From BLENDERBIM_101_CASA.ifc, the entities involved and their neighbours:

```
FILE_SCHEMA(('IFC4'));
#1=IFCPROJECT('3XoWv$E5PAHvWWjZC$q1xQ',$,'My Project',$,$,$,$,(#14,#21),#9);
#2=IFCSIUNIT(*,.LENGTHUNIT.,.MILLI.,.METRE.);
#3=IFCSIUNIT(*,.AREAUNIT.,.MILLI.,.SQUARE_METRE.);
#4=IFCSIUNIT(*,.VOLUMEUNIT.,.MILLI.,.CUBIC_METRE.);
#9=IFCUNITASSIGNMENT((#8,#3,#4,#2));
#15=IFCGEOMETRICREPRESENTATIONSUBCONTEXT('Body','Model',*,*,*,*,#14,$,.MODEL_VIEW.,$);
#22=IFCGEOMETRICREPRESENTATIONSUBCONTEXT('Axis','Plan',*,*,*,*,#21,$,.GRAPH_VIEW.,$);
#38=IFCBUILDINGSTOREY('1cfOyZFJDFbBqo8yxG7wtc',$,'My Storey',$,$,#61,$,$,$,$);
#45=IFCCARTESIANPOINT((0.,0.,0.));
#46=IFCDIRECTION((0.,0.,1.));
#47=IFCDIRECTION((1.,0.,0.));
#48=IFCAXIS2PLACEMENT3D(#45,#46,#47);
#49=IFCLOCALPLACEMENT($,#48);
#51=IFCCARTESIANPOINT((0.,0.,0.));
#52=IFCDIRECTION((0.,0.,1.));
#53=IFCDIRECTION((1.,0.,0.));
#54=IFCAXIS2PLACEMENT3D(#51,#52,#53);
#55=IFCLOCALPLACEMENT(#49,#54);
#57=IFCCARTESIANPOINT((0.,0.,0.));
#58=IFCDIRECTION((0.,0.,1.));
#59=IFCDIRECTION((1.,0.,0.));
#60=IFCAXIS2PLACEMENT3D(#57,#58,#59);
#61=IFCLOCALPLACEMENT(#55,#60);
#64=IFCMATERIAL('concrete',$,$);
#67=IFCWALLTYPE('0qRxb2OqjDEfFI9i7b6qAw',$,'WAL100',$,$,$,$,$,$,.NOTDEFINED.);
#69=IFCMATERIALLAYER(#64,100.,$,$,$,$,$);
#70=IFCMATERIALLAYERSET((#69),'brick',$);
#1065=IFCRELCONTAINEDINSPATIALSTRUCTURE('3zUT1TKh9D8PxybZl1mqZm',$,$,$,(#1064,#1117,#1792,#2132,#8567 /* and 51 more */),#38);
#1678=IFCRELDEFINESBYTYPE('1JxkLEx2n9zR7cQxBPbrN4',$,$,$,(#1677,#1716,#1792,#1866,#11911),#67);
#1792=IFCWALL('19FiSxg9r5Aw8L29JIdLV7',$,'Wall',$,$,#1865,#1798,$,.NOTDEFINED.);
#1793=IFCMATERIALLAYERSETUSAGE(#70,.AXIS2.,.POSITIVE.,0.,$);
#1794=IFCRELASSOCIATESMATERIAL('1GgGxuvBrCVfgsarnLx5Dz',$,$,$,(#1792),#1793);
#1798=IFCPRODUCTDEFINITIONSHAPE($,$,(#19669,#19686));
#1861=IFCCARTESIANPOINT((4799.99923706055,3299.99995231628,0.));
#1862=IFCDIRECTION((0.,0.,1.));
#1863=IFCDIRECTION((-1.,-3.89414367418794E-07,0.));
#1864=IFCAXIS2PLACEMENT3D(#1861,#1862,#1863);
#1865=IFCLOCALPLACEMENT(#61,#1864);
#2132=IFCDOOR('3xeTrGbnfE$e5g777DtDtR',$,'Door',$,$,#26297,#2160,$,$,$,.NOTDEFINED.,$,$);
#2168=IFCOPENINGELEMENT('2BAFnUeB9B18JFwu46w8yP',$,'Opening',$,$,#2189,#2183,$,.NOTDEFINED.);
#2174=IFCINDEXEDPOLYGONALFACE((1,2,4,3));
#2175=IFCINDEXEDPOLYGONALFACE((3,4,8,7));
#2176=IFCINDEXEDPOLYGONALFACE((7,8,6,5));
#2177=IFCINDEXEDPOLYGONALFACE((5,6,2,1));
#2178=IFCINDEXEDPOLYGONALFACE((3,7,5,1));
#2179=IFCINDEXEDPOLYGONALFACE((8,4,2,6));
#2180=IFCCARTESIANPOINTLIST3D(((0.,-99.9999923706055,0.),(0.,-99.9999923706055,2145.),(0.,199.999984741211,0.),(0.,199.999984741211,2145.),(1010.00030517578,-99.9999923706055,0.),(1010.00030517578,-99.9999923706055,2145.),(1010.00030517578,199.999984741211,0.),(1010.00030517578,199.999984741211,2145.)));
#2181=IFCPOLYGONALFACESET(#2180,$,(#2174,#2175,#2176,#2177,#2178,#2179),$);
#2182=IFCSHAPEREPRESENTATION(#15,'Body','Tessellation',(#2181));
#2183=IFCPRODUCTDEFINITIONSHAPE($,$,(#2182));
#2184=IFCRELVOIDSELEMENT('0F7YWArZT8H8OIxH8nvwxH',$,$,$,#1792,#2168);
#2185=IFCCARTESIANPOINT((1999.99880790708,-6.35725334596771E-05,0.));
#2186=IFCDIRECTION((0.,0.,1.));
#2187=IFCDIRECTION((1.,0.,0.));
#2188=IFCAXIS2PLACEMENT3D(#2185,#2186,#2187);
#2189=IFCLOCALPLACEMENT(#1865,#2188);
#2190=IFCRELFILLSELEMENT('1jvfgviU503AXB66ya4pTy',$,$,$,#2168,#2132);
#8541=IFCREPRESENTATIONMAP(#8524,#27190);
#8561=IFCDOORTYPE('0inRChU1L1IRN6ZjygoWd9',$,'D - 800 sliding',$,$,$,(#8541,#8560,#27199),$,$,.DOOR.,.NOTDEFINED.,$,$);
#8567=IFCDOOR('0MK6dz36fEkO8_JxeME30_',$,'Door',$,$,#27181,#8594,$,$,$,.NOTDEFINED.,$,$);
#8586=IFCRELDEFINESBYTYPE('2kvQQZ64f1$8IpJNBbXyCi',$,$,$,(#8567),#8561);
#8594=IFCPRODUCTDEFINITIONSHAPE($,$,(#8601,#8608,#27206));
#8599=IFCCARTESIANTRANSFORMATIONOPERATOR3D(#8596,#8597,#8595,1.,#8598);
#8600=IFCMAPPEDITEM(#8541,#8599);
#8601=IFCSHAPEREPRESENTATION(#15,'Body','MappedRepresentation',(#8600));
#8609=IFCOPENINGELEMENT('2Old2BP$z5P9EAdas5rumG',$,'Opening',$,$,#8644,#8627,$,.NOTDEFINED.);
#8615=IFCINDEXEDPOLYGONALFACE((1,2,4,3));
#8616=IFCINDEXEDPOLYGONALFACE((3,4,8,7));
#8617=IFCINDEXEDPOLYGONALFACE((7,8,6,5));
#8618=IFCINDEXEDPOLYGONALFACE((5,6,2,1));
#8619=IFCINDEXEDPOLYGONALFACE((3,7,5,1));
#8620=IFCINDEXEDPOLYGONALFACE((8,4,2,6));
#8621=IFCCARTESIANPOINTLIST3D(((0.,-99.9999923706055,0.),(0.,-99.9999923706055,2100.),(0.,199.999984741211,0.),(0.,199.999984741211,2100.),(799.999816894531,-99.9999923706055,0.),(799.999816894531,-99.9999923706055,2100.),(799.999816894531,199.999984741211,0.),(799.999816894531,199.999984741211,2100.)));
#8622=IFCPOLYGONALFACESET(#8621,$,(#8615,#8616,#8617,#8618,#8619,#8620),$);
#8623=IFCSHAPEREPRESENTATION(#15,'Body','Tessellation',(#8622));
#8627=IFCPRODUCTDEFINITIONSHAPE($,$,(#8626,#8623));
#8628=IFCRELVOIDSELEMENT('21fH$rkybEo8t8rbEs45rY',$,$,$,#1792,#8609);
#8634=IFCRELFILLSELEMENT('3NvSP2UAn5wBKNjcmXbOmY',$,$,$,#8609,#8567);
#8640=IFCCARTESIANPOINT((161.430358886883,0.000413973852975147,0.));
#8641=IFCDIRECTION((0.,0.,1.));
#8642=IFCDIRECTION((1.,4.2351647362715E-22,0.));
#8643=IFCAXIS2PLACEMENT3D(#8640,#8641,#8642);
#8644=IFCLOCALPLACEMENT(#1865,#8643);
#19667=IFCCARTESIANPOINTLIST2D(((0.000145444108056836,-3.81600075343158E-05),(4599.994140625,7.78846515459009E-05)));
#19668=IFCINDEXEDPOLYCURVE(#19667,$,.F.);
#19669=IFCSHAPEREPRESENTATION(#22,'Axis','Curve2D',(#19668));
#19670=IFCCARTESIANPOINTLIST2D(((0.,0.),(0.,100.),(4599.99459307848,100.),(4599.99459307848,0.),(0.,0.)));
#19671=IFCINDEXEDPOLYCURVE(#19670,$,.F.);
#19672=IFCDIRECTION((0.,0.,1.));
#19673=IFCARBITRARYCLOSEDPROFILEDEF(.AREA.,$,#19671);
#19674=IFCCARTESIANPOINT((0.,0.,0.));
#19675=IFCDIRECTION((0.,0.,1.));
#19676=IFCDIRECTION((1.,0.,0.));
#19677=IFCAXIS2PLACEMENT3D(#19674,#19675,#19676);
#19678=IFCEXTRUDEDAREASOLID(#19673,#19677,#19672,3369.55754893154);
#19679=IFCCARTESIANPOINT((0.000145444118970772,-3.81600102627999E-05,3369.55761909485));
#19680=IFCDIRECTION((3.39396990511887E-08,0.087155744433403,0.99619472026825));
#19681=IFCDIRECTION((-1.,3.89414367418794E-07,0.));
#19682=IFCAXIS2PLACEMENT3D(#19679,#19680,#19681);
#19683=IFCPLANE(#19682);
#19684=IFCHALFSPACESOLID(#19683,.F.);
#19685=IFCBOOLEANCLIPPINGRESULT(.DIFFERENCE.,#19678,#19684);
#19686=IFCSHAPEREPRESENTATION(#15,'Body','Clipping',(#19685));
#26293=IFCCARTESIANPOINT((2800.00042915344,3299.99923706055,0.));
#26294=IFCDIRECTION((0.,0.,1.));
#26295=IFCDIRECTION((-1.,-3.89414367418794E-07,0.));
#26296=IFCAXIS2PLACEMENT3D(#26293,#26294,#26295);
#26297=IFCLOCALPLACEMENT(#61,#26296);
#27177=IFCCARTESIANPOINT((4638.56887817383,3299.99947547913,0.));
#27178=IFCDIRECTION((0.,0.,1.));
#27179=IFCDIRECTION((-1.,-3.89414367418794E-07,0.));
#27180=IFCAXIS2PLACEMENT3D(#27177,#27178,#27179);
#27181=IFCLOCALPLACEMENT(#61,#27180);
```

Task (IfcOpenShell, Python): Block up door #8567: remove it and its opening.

```python
import ifcopenshell
import ifcopenshell.api.feature
import ifcopenshell.api.root
import ifcopenshell.geom
import ifcopenshell.util.shape

model = ifcopenshell.open("BLENDERBIM_101_CASA.ifc")
settings = ifcopenshell.geom.settings()


def volume(element):
    """Net volume in cubic metres, openings subtracted."""
    shape = ifcopenshell.geom.create_shape(settings, element)
    return ifcopenshell.util.shape.get_volume(shape.geometry)


door = model.by_guid("0MK6dz36fEkO8_JxeME30_")
opening = door.FillsVoids[0].RelatingOpeningElement
wall = opening.VoidsElements[0].RelatingBuildingElement
before = volume(wall)

ifcopenshell.api.root.remove_product(model, product=door)
ifcopenshell.api.feature.remove_feature(model, feature=opening)

after = volume(wall)

print(f"wall volume {before:.3f} -> {after:.3f} m3")

model.write("BLENDERBIM_101_CASA_edited.ifc")
```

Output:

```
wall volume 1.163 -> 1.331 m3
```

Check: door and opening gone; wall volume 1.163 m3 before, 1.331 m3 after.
